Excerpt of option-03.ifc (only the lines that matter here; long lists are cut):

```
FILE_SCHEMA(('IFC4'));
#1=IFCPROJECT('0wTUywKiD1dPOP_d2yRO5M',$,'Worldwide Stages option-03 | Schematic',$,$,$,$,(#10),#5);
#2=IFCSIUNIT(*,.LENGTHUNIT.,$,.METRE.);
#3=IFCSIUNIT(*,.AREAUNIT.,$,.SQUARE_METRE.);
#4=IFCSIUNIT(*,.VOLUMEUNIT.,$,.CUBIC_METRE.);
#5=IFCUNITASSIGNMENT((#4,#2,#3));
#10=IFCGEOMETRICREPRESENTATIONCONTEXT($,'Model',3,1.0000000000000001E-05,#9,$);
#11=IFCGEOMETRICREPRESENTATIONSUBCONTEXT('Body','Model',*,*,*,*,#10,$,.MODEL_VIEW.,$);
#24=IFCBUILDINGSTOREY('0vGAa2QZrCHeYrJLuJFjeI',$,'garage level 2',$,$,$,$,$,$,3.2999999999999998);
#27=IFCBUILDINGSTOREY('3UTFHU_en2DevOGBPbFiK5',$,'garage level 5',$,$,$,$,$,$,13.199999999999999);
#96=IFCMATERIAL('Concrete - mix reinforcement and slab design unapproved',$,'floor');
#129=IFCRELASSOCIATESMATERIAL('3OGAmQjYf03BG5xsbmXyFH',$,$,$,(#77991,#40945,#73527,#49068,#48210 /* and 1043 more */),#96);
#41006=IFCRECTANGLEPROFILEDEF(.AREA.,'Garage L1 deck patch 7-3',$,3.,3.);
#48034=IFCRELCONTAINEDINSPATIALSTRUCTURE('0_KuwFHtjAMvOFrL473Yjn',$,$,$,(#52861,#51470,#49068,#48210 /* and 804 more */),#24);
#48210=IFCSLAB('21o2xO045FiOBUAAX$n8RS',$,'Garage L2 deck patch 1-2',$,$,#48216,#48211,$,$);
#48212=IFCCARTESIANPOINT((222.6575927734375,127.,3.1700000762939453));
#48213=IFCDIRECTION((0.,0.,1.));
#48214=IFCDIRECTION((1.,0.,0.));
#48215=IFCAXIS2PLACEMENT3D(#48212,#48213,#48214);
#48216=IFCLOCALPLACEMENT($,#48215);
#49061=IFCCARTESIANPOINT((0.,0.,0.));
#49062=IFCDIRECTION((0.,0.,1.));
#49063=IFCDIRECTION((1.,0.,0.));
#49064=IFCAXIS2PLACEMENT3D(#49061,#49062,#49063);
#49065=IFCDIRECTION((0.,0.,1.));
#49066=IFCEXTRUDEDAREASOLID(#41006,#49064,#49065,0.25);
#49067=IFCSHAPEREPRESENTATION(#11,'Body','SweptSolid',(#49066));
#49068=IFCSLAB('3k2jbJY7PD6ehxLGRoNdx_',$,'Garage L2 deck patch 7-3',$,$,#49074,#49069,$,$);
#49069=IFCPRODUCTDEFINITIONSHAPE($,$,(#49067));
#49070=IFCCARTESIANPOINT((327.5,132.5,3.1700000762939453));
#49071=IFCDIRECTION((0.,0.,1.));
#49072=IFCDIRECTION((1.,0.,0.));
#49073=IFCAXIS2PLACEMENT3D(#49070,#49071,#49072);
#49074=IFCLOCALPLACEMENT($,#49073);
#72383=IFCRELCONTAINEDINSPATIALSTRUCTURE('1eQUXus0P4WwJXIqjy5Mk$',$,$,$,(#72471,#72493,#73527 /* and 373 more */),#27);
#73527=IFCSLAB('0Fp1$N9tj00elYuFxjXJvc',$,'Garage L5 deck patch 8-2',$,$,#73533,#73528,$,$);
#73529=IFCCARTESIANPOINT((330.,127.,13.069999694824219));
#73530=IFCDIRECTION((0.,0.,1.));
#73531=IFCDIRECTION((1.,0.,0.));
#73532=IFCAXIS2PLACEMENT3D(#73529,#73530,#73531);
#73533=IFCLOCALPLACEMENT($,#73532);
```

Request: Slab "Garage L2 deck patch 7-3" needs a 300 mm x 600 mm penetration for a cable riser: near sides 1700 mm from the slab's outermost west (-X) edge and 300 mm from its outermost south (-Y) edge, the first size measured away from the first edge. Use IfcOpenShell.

```python
import numpy as np
import ifcopenshell
import ifcopenshell.api.feature
import ifcopenshell.api.geometry
import ifcopenshell.api.root
import ifcopenshell.geom
import ifcopenshell.util.placement
import ifcopenshell.util.representation
import ifcopenshell.util.shape
import ifcopenshell.util.unit

model = ifcopenshell.open("option-03.ifc")
unit_scale = ifcopenshell.util.unit.calculate_unit_scale(model)
settings = ifcopenshell.geom.settings()


def volume(element):
    """Net volume in cubic metres, openings subtracted."""
    shape = ifcopenshell.geom.create_shape(settings, element)
    return ifcopenshell.util.shape.get_volume(shape.geometry)


slab = model.by_id(49068)
before = volume(slab)

# Extent in the slab's own axes, in metres. The edges named are its -X and -Y sides.
slab_shape = ifcopenshell.geom.create_shape(settings, slab)
vertices = ifcopenshell.util.shape.get_vertices(slab_shape.geometry)
x_min, y_min, bottom = vertices.min(axis=0)
top = vertices[:, 2].max()

opening = ifcopenshell.api.root.create_entity(model, ifc_class="IfcOpeningElement", name="Cable riser opening", predefined_type="OPENING")
context = ifcopenshell.util.representation.get_context(model, "Model", "Body", "MODEL_VIEW")
width, depth = 0.3, 0.6
outline = [(0.0, 0.0), (width, 0.0), (width, depth), (0.0, depth), (0.0, 0.0)]
# Overshoot both faces by 50 mm so the cut is clean.
shape = ifcopenshell.api.geometry.add_slab_representation(
    model, context=context, depth=top - bottom + 0.1, polyline=outline
)
ifcopenshell.api.geometry.assign_representation(model, product=opening, representation=shape)

matrix = ifcopenshell.util.placement.get_local_placement(slab.ObjectPlacement)
matrix[:, 3] = matrix @ np.append(np.array([x_min + 1.7, y_min + 0.3, bottom - 0.05]) / unit_scale, 1.0)
ifcopenshell.api.geometry.edit_object_placement(model, product=opening, matrix=matrix, is_si=False)
ifcopenshell.api.feature.add_feature(model, feature=opening, element=slab)

after = volume(slab)

print(f"slab volume {before:.3f} -> {after:.3f} m3")

model.write("option-03_rev.ifc")
```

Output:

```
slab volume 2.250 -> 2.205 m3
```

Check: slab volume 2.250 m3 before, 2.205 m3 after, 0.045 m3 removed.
